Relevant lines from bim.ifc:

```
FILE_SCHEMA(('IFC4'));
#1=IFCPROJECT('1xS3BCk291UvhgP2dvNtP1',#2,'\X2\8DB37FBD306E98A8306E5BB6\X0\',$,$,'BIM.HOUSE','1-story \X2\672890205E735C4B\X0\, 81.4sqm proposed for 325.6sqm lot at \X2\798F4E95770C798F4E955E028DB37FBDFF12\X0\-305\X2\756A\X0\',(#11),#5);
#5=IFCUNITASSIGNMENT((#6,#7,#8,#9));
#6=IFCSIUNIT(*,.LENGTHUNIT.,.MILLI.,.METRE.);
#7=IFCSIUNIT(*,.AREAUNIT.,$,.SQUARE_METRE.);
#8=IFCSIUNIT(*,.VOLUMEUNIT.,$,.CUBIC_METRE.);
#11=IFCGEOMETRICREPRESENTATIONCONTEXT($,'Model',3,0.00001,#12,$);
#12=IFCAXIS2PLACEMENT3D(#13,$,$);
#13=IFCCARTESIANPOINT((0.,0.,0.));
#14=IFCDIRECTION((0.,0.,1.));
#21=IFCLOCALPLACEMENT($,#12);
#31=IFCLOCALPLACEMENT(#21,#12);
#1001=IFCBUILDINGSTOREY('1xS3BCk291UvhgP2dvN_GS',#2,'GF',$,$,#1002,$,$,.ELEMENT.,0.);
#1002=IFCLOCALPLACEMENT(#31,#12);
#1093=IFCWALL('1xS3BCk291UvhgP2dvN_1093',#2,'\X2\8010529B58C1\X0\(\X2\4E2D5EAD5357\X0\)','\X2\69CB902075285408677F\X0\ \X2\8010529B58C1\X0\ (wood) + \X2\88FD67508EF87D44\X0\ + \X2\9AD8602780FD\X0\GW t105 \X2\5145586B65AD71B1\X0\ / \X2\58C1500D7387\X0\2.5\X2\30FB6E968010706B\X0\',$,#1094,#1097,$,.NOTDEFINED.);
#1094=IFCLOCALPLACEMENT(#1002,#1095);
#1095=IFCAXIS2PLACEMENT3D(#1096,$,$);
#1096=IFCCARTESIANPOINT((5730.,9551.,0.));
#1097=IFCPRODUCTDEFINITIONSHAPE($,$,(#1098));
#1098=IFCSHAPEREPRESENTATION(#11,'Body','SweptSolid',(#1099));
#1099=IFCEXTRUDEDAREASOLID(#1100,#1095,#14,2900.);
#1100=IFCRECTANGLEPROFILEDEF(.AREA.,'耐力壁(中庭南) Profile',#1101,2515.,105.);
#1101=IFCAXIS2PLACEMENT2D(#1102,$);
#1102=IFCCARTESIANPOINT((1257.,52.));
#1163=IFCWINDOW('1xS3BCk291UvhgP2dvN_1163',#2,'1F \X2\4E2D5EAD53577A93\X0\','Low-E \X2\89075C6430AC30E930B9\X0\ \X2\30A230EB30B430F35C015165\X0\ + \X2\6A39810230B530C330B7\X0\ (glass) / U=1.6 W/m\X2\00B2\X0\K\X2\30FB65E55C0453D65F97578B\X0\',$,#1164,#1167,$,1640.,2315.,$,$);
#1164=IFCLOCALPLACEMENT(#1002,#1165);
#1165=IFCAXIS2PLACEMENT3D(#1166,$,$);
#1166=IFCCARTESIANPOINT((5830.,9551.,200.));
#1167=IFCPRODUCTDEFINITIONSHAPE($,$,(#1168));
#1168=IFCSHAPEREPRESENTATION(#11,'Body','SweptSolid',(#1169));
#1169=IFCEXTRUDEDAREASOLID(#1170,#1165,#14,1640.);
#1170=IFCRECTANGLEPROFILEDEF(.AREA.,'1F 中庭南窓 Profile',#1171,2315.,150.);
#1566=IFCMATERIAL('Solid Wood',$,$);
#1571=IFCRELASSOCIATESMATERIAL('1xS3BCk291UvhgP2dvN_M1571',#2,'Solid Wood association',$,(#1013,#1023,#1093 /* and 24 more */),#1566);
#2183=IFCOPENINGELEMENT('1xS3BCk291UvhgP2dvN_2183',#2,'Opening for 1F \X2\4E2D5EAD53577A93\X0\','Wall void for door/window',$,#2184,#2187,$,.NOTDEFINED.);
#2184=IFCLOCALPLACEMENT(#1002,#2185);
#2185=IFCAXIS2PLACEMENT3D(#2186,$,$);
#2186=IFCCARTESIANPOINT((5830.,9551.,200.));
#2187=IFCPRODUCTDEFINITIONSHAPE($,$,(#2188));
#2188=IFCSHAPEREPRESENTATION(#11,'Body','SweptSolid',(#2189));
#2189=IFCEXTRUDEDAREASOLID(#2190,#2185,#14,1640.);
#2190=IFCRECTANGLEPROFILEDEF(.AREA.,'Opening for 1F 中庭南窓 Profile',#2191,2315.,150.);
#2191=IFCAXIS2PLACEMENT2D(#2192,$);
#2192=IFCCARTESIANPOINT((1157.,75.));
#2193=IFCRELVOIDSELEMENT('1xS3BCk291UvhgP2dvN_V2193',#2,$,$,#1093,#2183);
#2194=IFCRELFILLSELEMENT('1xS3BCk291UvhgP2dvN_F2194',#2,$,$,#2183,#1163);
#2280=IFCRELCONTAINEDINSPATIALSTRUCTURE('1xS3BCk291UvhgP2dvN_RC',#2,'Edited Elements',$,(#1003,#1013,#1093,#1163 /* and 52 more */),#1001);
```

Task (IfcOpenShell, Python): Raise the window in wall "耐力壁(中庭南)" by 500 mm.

```python
import numpy as np
import ifcopenshell
import ifcopenshell.api.geometry
import ifcopenshell.util.placement
import ifcopenshell.util.unit

model = ifcopenshell.open("bim.ifc")
unit_scale = ifcopenshell.util.unit.calculate_unit_scale(model)

window = model.by_id(1163)
opening = window.FillsVoids[0].RelatingOpeningElement
dz = 0.5 / unit_scale

shift = np.array([0.0, 0.0, dz])
# The window is not placed relative to its opening, so move both.
for product in (opening, window):
    matrix = ifcopenshell.util.placement.get_local_placement(product.ObjectPlacement)
    matrix[:3, 3] += shift
    ifcopenshell.api.geometry.edit_object_placement(model, product=product, matrix=matrix, is_si=False)

print(f"moved by {dz * unit_scale:+.3f} m")

model.write("bim-out.ifc")
```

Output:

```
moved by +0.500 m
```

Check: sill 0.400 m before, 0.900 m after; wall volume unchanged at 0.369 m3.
